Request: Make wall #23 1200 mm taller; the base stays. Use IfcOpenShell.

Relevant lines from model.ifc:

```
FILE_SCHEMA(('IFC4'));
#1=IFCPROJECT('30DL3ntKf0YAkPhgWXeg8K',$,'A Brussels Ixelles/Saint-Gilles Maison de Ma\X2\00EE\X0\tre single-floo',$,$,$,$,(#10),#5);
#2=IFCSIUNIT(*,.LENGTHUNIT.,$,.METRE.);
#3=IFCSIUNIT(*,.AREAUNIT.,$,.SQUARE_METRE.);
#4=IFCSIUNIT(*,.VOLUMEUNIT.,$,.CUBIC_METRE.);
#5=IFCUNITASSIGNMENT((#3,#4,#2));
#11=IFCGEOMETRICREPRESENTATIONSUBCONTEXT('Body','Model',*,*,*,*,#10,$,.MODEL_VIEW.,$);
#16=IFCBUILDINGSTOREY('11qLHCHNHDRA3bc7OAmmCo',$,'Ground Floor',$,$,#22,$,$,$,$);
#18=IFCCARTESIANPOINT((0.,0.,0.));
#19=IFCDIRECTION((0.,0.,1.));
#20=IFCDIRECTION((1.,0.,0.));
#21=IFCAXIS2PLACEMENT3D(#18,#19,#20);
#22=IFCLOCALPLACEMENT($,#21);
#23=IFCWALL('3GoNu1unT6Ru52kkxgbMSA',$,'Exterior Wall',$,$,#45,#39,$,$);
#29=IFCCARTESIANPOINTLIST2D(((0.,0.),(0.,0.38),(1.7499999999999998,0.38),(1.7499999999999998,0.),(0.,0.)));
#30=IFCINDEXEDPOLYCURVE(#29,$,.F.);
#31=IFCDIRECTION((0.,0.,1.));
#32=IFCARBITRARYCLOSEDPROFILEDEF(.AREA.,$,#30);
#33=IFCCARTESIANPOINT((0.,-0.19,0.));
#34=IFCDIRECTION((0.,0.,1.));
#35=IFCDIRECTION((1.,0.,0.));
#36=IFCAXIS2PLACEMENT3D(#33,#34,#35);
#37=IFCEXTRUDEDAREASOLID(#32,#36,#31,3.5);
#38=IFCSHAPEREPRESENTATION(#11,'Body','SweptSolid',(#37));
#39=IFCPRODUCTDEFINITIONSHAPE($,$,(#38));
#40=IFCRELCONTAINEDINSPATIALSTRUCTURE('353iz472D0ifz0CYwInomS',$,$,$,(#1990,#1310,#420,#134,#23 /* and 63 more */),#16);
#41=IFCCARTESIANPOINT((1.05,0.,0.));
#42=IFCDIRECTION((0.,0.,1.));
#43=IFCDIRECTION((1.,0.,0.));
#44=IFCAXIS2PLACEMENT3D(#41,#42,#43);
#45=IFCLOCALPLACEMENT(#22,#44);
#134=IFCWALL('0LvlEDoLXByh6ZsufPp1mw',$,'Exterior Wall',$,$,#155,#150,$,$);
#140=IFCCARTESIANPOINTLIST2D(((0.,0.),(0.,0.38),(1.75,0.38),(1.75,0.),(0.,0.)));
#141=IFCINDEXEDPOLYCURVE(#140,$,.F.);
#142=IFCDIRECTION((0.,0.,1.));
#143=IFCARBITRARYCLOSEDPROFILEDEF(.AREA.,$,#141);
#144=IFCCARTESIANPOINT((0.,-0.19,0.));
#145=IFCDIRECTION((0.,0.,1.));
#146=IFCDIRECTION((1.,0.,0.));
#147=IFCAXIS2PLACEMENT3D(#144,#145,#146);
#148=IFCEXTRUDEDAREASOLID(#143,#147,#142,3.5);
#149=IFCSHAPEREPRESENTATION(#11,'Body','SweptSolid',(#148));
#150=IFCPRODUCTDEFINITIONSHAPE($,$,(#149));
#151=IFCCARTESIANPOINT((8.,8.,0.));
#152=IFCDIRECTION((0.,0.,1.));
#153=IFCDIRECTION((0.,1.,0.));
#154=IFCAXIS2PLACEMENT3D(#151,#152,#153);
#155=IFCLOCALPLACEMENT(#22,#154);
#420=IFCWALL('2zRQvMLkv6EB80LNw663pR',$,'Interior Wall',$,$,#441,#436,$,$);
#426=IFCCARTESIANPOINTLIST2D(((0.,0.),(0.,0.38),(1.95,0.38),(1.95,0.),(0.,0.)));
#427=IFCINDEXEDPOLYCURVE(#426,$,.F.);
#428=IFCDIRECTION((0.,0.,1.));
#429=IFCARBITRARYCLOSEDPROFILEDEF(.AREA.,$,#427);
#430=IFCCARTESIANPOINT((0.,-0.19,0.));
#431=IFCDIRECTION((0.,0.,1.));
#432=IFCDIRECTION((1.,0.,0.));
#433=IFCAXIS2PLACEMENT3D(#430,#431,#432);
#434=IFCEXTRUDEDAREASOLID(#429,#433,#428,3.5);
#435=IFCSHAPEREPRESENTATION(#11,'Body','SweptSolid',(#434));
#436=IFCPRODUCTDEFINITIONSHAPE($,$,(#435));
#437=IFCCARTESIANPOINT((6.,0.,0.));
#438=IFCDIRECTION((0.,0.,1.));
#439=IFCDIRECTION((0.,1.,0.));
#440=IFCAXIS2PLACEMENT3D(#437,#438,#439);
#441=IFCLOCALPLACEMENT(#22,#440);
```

```python
import ifcopenshell
import ifcopenshell.geom
import ifcopenshell.util.representation
import ifcopenshell.util.shape
import ifcopenshell.util.unit

model = ifcopenshell.open("model.ifc")
unit_scale = ifcopenshell.util.unit.calculate_unit_scale(model)
settings = ifcopenshell.geom.settings()


def volume(element):
    """Net volume in cubic metres, openings subtracted."""
    shape = ifcopenshell.geom.create_shape(settings, element)
    return ifcopenshell.util.shape.get_volume(shape.geometry)


wall = model.by_id(23)
before = volume(wall)

body = ifcopenshell.util.representation.get_representation(wall, "Model", "Body")
solid = body.Items[0]
old_height = solid.Depth
solid.Depth += 1.2 / unit_scale
after = volume(wall)

print(f"height {old_height:g} -> {solid.Depth:g}, volume {before:.3f} -> {after:.3f} m3")

model.write("model_edited.ifc")
```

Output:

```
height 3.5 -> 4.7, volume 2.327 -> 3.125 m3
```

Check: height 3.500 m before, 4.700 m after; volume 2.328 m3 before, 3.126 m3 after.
